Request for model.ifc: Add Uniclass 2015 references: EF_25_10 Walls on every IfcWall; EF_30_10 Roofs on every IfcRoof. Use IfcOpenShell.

First a look at what the model holds.

```python
import ifcopenshell

model = ifcopenshell.open("model.ifc")
print(model.schema)
print("classifications:", [c.Name for c in model.by_type("IfcClassification")])
for ifc_class in ("IfcDoor", "IfcRoof", "IfcStair", "IfcWall", "IfcWindow"):
    print(ifc_class, len(model.by_type(ifc_class)))
```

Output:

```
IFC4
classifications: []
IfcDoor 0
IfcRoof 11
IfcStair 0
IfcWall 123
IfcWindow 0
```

```python
import ifcopenshell
import ifcopenshell.api.classification

model = ifcopenshell.open("model.ifc")

system = ifcopenshell.api.classification.add_classification(model, classification="Uniclass 2015")

codes = {
    "IfcWall": ("EF_25_10", "Walls"),
    "IfcRoof": ("EF_30_10", "Roofs"),
}
for ifc_class, (code, name) in codes.items():
    products = model.by_type(ifc_class)
    ifcopenshell.api.classification.add_reference(
        model, products=products, classification=system, identification=code, name=name
    )
    print(code, len(products))

model.write("model-out.ifc")
```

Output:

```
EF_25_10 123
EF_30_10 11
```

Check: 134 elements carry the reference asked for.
